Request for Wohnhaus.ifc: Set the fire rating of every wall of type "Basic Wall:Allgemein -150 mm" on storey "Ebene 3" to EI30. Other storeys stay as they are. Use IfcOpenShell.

First a look at what the model holds.

```python
import ifcopenshell
import ifcopenshell.util.element

model = ifcopenshell.open("Wohnhaus.ifc")
print(model.schema)
storey = next(s for s in model.by_type("IfcBuildingStorey") if s.Name == "Ebene 3")
walls = [e for e in ifcopenshell.util.element.get_decomposition(storey) if e.is_a("IfcWall")]
seen = {}
for e in walls:
    element_type = ifcopenshell.util.element.get_type(e)
    key = (element_type.Name if element_type != e and element_type else None, ifcopenshell.util.element.get_pset(e, "Pset_WallCommon", "FireRating"))
    seen[key] = seen.get(key, 0) + 1
for (name, value), count in sorted(seen.items(), key=str):
    print(count, "x", name, "|", value)
```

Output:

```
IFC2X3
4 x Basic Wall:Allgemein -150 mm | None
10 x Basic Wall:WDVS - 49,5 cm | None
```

```python
import ifcopenshell
import ifcopenshell.api.pset
import ifcopenshell.util.element

model = ifcopenshell.open("Wohnhaus.ifc")

storey = next(s for s in model.by_type("IfcBuildingStorey") if s.Name == "Ebene 3")
walls = [e for e in ifcopenshell.util.element.get_decomposition(storey) if e.is_a("IfcWall")]

count = 0
for e in walls:
    element_type = ifcopenshell.util.element.get_type(e)
    if element_type in (None, e) or element_type.Name != "Basic Wall:Allgemein -150 mm":
        continue
    # add_pset returns the element's existing set when there is one.
    pset = ifcopenshell.api.pset.add_pset(model, product=e, name="Pset_WallCommon")
    ifcopenshell.api.pset.edit_pset(model, pset=pset, properties={"FireRating": "EI30"})
    count += 1

print(count, "walls updated")

model.write("Wohnhaus_edited.ifc")
```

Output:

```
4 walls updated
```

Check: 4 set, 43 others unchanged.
